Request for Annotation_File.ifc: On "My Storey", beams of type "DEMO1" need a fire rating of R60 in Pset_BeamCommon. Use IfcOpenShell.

First a look at what the model holds.

```python
import ifcopenshell
import ifcopenshell.util.element

model = ifcopenshell.open("Annotation_File.ifc")
print(model.schema)
storey = next(s for s in model.by_type("IfcBuildingStorey") if s.Name == "My Storey")
beams = [e for e in ifcopenshell.util.element.get_decomposition(storey) if e.is_a("IfcBeam")]
seen = {}
for e in beams:
    element_type = ifcopenshell.util.element.get_type(e)
    key = (element_type.Name if element_type != e and element_type else None, ifcopenshell.util.element.get_pset(e, "Pset_BeamCommon", "FireRating"))
    seen[key] = seen.get(key, 0) + 1
for (name, value), count in sorted(seen.items(), key=str):
    print(count, "x", name, "|", value)
```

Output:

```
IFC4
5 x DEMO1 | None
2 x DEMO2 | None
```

```python
import ifcopenshell
import ifcopenshell.api.pset
import ifcopenshell.util.element

model = ifcopenshell.open("Annotation_File.ifc")

storey = next(s for s in model.by_type("IfcBuildingStorey") if s.Name == "My Storey")
beams = [e for e in ifcopenshell.util.element.get_decomposition(storey) if e.is_a("IfcBeam")]

count = 0
for e in beams:
    element_type = ifcopenshell.util.element.get_type(e)
    if element_type in (None, e) or element_type.Name != "DEMO1":
        continue
    # add_pset returns the element's existing set when there is one.
    pset = ifcopenshell.api.pset.add_pset(model, product=e, name="Pset_BeamCommon")
    ifcopenshell.api.pset.edit_pset(model, pset=pset, properties={"FireRating": "R60"})
    count += 1

print(count, "beams updated")

model.write("Annotation_File_updated.ifc")
```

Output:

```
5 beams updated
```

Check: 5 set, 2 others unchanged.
